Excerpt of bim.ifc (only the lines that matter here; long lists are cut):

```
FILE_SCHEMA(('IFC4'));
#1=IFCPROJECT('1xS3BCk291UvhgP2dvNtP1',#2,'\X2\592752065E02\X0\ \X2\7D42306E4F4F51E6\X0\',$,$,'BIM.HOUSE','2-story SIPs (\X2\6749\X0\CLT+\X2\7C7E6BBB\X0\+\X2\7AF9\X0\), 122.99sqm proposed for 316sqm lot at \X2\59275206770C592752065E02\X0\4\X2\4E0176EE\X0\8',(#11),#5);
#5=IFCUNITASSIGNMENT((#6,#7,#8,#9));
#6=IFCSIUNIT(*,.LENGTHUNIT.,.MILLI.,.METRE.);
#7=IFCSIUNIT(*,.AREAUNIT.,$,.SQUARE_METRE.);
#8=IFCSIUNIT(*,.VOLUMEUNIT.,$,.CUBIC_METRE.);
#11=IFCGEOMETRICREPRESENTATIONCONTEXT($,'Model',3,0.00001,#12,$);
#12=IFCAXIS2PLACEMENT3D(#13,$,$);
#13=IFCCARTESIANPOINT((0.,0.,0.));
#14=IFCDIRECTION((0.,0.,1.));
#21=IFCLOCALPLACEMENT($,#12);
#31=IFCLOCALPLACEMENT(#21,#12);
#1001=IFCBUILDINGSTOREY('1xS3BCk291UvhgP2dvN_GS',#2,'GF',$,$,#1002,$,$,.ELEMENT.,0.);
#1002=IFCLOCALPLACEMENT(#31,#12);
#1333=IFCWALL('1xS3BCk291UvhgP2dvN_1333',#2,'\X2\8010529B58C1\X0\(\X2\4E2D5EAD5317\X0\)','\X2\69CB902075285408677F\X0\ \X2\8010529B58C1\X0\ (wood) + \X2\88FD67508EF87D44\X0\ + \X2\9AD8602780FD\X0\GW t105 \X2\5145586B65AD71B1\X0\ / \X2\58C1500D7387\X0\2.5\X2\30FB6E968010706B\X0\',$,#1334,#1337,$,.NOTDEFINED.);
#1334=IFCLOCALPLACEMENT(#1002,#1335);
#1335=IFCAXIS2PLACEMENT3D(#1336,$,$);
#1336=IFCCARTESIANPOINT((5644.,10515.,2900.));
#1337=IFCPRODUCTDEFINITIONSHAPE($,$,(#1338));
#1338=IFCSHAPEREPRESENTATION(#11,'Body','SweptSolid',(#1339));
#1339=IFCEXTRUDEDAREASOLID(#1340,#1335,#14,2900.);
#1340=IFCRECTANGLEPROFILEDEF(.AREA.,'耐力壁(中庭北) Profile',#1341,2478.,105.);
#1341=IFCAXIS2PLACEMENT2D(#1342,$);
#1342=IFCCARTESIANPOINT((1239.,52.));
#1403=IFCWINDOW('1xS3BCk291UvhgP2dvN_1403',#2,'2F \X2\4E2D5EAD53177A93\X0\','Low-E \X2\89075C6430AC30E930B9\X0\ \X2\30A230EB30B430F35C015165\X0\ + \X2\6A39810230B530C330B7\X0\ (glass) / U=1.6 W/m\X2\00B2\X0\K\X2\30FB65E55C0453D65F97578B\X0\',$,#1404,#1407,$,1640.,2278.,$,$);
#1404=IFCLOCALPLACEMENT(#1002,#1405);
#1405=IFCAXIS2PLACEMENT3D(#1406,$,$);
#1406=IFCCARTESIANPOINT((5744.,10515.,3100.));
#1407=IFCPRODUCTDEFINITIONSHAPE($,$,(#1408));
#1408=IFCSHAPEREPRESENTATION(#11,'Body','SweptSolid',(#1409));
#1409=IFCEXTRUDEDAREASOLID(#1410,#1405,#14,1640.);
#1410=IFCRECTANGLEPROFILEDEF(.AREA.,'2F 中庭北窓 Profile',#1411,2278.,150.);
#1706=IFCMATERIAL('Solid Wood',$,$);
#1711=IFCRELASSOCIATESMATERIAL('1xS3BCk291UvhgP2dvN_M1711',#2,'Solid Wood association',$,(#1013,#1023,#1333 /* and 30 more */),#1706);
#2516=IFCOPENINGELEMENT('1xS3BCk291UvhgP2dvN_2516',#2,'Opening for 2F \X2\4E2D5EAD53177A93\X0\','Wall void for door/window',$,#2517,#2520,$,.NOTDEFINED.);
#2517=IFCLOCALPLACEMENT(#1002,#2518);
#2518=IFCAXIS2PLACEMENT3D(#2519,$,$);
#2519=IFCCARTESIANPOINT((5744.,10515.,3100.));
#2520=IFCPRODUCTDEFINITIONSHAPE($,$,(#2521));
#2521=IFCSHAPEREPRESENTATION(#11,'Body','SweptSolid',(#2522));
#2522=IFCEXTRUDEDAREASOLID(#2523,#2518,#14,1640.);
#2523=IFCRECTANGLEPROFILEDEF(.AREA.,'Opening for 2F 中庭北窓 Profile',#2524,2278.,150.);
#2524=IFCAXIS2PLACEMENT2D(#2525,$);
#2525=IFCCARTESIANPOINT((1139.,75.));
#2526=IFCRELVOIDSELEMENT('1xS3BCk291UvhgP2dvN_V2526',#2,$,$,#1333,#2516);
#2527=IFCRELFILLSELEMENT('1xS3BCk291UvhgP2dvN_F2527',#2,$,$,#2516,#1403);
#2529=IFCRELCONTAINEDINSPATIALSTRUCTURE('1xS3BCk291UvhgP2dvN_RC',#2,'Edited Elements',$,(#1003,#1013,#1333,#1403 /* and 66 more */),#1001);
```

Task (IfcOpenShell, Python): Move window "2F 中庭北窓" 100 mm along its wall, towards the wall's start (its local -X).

```python
import ifcopenshell
import ifcopenshell.api.geometry
import ifcopenshell.util.placement

model = ifcopenshell.open("bim.ifc")

window = model.by_guid("1xS3BCk291UvhgP2dvN_1403")
opening = window.FillsVoids[0].RelatingOpeningElement
wall = opening.VoidsElements[0].RelatingBuildingElement

wall_matrix = ifcopenshell.util.placement.get_local_placement(wall.ObjectPlacement)
shift = wall_matrix[:3, 0] * -100.0
before = ifcopenshell.util.placement.get_local_placement(window.ObjectPlacement)[:3, 3].copy()

# The window is not placed relative to its opening, so move both.
for product in (opening, window):
    matrix = ifcopenshell.util.placement.get_local_placement(product.ObjectPlacement)
    matrix[:3, 3] += shift
    ifcopenshell.api.geometry.edit_object_placement(model, product=product, matrix=matrix, is_si=False)

after = ifcopenshell.util.placement.get_local_placement(window.ObjectPlacement)[:3, 3]
print("window moved by", (after - before).round(3) + 0.0)

model.write("bim-out.ifc")
```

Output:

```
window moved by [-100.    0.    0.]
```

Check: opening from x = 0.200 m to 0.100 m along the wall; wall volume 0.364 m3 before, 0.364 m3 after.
